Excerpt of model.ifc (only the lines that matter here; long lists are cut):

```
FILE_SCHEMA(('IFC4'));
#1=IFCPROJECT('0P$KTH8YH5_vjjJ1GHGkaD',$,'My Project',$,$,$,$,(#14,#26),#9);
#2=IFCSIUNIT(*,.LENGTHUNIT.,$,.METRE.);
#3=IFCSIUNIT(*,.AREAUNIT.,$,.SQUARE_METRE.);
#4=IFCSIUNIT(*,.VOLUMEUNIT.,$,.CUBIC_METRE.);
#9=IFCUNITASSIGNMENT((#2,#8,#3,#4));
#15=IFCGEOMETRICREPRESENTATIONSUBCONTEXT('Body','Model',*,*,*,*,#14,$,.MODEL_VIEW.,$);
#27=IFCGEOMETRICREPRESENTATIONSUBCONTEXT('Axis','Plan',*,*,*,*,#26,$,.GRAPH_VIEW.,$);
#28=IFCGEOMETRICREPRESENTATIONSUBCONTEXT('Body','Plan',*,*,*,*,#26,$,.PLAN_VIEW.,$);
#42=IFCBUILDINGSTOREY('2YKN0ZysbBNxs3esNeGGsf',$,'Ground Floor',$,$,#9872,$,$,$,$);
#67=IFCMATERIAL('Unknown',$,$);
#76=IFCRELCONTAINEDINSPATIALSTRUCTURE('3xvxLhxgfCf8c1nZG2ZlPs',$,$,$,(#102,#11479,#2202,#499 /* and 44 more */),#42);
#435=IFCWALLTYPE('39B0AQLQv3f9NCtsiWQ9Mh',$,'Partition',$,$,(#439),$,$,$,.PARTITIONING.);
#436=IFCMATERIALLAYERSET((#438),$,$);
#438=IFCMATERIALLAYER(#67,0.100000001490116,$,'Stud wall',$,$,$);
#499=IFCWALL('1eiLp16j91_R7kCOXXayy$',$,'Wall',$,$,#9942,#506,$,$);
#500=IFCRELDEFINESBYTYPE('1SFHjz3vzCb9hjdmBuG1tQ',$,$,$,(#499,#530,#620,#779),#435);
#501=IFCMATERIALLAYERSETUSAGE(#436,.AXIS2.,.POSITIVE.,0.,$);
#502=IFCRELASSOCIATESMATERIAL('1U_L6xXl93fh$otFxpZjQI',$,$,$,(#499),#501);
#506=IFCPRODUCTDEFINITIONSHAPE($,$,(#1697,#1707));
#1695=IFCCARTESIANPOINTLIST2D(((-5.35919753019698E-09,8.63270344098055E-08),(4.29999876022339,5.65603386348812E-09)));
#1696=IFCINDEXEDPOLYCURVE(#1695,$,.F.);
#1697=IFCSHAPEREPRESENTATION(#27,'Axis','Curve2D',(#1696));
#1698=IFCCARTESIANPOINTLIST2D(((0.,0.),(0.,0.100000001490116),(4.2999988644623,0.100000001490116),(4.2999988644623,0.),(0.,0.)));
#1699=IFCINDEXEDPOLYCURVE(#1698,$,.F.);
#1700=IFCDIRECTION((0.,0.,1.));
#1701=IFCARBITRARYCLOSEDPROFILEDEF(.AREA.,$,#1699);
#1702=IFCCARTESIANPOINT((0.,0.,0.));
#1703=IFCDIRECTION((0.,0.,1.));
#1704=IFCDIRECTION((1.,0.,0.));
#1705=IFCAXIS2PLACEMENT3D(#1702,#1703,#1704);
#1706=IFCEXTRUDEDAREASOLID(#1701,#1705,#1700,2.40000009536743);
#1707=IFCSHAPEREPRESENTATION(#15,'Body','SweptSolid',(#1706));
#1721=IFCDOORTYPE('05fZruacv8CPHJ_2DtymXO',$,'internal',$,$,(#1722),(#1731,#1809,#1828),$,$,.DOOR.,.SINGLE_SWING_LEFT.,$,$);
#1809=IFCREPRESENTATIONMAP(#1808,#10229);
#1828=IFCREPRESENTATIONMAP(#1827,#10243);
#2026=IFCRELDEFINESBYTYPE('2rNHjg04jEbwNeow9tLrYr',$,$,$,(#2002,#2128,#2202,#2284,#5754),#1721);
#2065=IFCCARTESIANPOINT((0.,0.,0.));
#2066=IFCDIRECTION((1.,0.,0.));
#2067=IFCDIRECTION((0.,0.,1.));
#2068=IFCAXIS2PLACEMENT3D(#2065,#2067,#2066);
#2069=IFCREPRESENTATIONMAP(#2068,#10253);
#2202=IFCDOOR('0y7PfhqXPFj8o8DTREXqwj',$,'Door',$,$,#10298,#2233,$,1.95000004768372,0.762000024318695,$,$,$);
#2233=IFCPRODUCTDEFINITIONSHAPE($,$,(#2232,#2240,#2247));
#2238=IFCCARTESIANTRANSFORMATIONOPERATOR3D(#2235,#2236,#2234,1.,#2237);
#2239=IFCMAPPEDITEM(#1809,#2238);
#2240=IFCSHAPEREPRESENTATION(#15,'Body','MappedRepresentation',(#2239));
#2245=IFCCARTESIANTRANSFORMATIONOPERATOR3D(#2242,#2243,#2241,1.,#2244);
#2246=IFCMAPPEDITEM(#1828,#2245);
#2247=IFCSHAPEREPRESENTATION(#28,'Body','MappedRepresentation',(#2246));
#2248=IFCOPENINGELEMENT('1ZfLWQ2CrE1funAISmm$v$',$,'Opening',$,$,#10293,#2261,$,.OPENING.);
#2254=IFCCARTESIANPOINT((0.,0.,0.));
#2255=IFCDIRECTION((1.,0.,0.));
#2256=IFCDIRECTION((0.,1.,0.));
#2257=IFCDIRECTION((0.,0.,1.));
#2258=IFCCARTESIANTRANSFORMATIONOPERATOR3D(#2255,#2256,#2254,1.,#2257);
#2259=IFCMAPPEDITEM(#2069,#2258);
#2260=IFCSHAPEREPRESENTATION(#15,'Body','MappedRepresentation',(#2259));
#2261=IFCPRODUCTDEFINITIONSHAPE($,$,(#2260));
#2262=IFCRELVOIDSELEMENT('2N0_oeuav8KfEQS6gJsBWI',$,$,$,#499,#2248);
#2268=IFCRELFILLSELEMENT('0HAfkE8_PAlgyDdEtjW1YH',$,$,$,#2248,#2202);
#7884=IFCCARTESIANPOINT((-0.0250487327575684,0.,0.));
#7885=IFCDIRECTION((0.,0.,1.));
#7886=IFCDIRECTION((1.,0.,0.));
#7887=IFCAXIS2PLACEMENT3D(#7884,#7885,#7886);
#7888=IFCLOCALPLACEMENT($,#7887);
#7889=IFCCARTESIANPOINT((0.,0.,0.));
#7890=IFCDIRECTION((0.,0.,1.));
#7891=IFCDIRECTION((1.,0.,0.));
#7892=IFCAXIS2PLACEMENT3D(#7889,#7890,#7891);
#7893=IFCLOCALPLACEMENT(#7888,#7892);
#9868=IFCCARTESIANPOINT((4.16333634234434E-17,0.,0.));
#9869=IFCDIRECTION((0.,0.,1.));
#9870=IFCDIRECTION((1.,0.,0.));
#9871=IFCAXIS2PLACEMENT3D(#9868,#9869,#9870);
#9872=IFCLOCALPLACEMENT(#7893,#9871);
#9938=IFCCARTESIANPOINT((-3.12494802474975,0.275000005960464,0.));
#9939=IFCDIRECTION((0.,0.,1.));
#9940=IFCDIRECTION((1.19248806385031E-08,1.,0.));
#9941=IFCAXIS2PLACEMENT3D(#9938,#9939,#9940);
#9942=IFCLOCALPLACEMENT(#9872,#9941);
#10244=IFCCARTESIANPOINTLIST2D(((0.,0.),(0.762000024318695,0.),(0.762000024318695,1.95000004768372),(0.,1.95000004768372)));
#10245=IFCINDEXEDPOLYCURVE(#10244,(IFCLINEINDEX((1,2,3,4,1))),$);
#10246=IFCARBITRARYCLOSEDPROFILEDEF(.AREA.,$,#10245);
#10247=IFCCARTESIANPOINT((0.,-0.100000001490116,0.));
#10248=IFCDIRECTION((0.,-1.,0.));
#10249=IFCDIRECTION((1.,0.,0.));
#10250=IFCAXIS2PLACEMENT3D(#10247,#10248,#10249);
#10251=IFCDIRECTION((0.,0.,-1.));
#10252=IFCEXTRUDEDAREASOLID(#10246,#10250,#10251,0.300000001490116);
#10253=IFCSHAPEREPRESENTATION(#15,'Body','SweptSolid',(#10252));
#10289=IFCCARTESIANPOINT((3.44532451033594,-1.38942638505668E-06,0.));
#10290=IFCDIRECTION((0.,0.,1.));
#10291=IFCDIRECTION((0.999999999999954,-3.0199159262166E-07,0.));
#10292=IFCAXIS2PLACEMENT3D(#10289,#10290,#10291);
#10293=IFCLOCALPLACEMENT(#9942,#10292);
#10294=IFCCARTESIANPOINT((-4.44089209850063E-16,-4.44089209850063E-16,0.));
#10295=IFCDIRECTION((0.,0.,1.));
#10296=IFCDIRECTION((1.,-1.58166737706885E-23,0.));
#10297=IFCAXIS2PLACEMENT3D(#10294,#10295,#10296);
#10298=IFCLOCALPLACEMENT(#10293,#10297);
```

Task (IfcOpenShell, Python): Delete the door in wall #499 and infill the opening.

```python
import ifcopenshell
import ifcopenshell.api.feature
import ifcopenshell.api.root
import ifcopenshell.geom
import ifcopenshell.util.shape

model = ifcopenshell.open("model.ifc")
settings = ifcopenshell.geom.settings()


def volume(element):
    """Net volume in cubic metres, openings subtracted."""
    shape = ifcopenshell.geom.create_shape(settings, element)
    return ifcopenshell.util.shape.get_volume(shape.geometry)


door = model.by_id(2202)
opening = door.FillsVoids[0].RelatingOpeningElement
wall = opening.VoidsElements[0].RelatingBuildingElement
before = volume(wall)

ifcopenshell.api.root.remove_product(model, product=door)
ifcopenshell.api.feature.remove_feature(model, feature=opening)

after = volume(wall)

print(f"wall volume {before:.3f} -> {after:.3f} m3")

model.write("model_edited.ifc")
```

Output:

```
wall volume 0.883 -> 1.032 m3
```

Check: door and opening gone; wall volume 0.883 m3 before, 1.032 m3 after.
